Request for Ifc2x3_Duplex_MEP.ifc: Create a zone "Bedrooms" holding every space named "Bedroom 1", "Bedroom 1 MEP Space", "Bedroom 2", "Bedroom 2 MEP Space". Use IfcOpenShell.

First a look at what the model holds.

```python
import ifcopenshell

model = ifcopenshell.open("Ifc2x3_Duplex_MEP.ifc")
print(model.schema)
seen = {}
for space in model.by_type("IfcSpace"):
    seen[space.LongName] = seen.get(space.LongName, 0) + 1
for name, count in sorted(seen.items(), key=str):
    print(count, "x", name)
print("zones:", [z.Name for z in model.by_type("IfcZone")][:20])
```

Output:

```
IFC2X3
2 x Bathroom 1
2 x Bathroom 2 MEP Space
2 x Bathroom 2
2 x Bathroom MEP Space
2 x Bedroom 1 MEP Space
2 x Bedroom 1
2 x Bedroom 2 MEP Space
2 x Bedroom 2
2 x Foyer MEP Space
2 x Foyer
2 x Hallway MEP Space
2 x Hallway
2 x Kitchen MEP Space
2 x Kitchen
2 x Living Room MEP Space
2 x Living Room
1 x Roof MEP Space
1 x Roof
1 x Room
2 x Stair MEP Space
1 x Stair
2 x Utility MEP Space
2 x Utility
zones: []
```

```python
import ifcopenshell
import ifcopenshell.api.group
import ifcopenshell.api.root

model = ifcopenshell.open("Ifc2x3_Duplex_MEP.ifc")

names = {"Bedroom 1", "Bedroom 1 MEP Space", "Bedroom 2", "Bedroom 2 MEP Space"}
spaces = [s for s in model.by_type("IfcSpace") if s.LongName in names]

zone = ifcopenshell.api.root.create_entity(model, ifc_class="IfcZone", name="Bedrooms")
ifcopenshell.api.group.assign_group(model, products=spaces, group=zone)
print(len(spaces), "spaces in", zone.Name)

model.write("Ifc2x3_Duplex_MEP_updated.ifc")
```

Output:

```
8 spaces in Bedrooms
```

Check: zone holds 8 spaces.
